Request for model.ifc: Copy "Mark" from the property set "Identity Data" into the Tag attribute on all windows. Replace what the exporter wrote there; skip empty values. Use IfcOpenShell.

First a look at what the model holds.

```python
import ifcopenshell
import ifcopenshell.util.element

model = ifcopenshell.open("model.ifc")
print(model.schema)
windows = model.by_type("IfcWindow")
print(len(windows), "windows")
for e in windows[:8]:
    source = ifcopenshell.util.element.get_pset(e, "Identity Data", "Mark")
    target = e.Tag
    print(e.id(), repr(source), repr(target), sep=" | ")
```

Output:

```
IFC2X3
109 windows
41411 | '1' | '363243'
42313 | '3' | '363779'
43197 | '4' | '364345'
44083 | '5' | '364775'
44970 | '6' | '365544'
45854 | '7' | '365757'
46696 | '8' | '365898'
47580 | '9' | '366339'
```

```python
import ifcopenshell
import ifcopenshell.util.element

model = ifcopenshell.open("model.ifc")

count = 0
for e in model.by_type("IfcWindow"):
    value = ifcopenshell.util.element.get_pset(e, "Identity Data", "Mark")
    current = e.Tag
    if not value or not value.strip() or current == value:
        continue
    e.Tag = value
    count += 1

print(count, "windows updated")

model.write("model_edited.ifc")
```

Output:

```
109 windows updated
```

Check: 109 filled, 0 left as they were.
